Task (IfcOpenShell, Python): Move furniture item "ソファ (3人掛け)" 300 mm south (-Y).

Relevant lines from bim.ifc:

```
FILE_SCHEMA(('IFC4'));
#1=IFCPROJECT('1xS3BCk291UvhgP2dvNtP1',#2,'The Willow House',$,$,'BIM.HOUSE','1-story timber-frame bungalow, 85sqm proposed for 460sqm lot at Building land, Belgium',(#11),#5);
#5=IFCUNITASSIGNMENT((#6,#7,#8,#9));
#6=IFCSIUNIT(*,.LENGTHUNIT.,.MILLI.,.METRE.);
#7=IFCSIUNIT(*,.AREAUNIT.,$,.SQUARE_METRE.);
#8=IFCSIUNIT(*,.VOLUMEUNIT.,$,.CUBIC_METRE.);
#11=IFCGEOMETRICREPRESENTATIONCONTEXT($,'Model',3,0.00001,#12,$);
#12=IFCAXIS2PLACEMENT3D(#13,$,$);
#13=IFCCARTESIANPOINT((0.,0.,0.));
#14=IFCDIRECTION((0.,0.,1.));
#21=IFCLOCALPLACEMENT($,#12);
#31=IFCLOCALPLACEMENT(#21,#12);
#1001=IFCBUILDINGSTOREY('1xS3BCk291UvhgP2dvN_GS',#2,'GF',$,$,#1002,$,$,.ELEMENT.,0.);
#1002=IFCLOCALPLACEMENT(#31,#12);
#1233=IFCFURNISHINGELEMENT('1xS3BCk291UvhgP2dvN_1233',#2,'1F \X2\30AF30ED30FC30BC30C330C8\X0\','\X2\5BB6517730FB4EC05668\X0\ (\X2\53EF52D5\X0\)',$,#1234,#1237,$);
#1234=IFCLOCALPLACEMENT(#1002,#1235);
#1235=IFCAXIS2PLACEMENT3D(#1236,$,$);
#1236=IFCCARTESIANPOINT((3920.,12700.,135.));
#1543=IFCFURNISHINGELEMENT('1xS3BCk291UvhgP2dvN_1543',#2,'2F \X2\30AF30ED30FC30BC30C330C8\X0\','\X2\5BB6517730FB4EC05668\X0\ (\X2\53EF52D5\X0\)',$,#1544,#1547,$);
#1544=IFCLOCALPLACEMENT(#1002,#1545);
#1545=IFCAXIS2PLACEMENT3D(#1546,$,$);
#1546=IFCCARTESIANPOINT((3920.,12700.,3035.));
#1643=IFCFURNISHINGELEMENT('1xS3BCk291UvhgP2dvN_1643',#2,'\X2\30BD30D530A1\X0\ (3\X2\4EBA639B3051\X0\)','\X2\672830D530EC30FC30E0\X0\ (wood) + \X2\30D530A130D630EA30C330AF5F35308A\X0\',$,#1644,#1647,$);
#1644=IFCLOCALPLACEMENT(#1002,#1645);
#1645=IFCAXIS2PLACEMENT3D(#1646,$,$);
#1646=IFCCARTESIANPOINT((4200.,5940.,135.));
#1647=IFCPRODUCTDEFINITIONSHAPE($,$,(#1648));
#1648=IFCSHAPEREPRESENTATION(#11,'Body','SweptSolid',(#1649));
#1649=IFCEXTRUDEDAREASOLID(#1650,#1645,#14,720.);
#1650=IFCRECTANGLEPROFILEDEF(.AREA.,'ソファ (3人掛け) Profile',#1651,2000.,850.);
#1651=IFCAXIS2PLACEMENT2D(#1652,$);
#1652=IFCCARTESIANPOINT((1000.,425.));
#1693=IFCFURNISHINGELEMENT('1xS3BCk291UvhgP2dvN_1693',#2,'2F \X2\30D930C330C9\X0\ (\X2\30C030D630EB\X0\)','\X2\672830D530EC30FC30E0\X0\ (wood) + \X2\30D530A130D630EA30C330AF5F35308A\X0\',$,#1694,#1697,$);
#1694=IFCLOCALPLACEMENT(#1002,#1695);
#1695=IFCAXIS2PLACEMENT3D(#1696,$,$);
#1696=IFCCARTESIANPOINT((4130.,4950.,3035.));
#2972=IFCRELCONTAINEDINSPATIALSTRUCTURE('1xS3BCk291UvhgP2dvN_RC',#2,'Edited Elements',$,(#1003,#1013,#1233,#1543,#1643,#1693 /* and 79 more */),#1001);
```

```python
import ifcopenshell
import ifcopenshell.api.geometry
import ifcopenshell.util.placement
import ifcopenshell.util.unit

model = ifcopenshell.open("bim.ifc")
unit_scale = ifcopenshell.util.unit.calculate_unit_scale(model)

item = model.by_guid("1xS3BCk291UvhgP2dvN_1643")
matrix = ifcopenshell.util.placement.get_local_placement(item.ObjectPlacement)
matrix[1, 3] -= 0.3 / unit_scale
ifcopenshell.api.geometry.edit_object_placement(model, product=item, matrix=matrix, is_si=False)

print(ifcopenshell.util.placement.get_local_placement(item.ObjectPlacement).round(3) + 0.0)

model.write("bim_edited.ifc")
```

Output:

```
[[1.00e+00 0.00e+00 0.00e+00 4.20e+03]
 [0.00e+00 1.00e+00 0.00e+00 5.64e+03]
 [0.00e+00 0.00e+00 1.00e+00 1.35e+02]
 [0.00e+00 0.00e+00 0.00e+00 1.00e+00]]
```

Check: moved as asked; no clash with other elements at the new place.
